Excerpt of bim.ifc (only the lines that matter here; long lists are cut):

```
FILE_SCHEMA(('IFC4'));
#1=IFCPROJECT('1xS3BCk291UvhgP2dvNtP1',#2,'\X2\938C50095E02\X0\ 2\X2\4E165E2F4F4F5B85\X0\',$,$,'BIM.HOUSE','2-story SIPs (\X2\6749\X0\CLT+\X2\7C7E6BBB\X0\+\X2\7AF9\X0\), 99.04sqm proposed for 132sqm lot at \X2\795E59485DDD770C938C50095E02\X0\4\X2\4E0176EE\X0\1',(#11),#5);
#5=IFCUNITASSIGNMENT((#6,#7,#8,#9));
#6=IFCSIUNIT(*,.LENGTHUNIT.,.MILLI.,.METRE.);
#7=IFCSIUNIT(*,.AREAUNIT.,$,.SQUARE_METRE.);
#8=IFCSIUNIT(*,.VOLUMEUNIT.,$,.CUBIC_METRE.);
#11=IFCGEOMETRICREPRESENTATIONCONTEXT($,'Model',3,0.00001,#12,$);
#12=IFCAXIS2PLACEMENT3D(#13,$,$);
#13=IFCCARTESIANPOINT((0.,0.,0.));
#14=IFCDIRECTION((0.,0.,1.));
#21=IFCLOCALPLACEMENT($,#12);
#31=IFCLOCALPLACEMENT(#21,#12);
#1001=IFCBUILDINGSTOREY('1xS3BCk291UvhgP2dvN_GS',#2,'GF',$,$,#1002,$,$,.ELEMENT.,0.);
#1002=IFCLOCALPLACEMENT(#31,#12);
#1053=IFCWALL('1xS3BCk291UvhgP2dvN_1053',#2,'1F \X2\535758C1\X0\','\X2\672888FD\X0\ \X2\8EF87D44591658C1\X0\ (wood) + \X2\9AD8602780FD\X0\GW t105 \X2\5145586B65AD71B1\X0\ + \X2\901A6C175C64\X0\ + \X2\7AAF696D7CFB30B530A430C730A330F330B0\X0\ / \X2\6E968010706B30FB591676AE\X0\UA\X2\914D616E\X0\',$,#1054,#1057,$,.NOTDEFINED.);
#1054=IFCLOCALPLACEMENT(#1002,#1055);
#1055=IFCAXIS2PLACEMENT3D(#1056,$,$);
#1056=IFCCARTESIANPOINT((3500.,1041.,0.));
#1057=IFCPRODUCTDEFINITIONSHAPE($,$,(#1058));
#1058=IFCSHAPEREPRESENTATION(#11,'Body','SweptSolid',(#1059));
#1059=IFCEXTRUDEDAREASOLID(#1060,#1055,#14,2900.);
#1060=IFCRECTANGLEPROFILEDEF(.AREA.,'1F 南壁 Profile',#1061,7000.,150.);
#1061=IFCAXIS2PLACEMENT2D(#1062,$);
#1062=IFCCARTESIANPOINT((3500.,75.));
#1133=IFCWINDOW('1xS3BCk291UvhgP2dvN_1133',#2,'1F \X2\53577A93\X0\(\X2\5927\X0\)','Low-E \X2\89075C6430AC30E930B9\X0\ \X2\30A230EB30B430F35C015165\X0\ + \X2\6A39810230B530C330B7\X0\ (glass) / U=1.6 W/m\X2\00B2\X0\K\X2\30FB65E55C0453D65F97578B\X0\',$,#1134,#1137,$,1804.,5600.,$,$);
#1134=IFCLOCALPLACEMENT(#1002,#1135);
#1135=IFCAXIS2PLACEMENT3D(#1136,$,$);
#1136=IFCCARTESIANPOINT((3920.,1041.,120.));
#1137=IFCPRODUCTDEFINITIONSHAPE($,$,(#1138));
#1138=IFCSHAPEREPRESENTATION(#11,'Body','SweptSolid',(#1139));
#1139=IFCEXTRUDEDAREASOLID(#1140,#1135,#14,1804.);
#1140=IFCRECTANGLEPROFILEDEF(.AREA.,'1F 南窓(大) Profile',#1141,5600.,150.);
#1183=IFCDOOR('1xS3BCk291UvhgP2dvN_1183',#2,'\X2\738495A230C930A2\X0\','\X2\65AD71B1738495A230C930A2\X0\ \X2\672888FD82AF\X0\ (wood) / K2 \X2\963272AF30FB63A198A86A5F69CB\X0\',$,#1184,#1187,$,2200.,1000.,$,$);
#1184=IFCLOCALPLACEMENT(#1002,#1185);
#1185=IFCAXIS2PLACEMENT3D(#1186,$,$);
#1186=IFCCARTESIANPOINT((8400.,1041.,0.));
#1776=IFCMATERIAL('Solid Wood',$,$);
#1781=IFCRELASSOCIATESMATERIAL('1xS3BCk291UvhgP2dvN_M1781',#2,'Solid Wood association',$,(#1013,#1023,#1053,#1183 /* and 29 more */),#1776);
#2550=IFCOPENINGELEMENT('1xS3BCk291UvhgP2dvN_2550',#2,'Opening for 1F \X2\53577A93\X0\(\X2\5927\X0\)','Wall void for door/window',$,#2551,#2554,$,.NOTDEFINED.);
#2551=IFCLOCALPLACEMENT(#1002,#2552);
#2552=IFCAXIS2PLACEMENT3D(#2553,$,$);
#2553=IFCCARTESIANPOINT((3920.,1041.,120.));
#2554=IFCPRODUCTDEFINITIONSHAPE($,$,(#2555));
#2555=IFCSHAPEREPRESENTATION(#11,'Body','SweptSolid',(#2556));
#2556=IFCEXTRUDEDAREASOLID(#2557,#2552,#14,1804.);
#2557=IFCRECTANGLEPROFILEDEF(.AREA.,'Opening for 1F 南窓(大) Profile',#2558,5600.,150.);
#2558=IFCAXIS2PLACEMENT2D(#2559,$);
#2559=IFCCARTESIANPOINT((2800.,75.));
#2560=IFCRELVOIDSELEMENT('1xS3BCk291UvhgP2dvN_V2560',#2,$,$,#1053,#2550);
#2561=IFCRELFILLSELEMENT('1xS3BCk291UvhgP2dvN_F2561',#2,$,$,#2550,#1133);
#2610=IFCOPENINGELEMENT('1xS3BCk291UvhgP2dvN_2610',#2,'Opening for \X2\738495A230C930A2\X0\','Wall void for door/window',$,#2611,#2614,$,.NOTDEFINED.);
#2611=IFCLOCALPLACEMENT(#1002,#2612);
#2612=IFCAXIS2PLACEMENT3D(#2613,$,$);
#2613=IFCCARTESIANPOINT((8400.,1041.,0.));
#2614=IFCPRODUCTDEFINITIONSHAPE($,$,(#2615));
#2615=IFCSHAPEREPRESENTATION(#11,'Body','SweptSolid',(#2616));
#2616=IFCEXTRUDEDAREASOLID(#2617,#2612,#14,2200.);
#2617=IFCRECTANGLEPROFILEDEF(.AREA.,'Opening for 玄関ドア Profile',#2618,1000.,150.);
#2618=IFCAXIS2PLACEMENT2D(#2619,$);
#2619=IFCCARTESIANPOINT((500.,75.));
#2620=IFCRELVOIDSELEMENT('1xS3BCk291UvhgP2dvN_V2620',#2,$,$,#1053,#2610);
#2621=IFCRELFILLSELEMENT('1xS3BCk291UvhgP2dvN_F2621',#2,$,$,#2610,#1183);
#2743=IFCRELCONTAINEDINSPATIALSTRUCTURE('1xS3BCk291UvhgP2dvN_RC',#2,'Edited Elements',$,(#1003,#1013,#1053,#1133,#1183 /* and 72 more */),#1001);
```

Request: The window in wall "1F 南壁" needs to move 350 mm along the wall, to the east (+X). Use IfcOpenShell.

```python
import ifcopenshell
import ifcopenshell.api.geometry
import ifcopenshell.util.placement
import ifcopenshell.util.unit

model = ifcopenshell.open("bim.ifc")
unit_scale = ifcopenshell.util.unit.calculate_unit_scale(model)

window = model.by_guid("1xS3BCk291UvhgP2dvN_1133")
opening = window.FillsVoids[0].RelatingOpeningElement
wall = opening.VoidsElements[0].RelatingBuildingElement

wall_matrix = ifcopenshell.util.placement.get_local_placement(wall.ObjectPlacement)
shift = wall_matrix[:3, 0] * 0.35 / unit_scale
before = ifcopenshell.util.placement.get_local_placement(window.ObjectPlacement)[:3, 3].copy()

# The window is not placed relative to its opening, so move both.
for product in (opening, window):
    matrix = ifcopenshell.util.placement.get_local_placement(product.ObjectPlacement)
    matrix[:3, 3] += shift
    ifcopenshell.api.geometry.edit_object_placement(model, product=product, matrix=matrix, is_si=False)

after = ifcopenshell.util.placement.get_local_placement(window.ObjectPlacement)[:3, 3]
print("window moved by", (after - before).round(3) + 0.0)

model.write("bim_updated.ifc")
```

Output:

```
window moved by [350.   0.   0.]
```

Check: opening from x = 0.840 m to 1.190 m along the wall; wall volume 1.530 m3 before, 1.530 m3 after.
